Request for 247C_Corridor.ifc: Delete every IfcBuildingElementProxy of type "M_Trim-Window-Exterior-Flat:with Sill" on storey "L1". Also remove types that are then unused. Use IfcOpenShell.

First a look at what the model holds.

```python
import ifcopenshell
import ifcopenshell.util.element

model = ifcopenshell.open("247C_Corridor.ifc")
print(model.schema)
storey = next(s for s in model.by_type("IfcBuildingStorey") if s.Name == "L1")
proxies = [e for e in ifcopenshell.util.element.get_decomposition(storey) if e.is_a("IfcBuildingElementProxy")]
seen = {}
for e in proxies:
    element_type = ifcopenshell.util.element.get_type(e)
    name = element_type.Name if element_type not in (None, e) else None
    seen[name] = seen.get(name, 0) + 1
for name, count in sorted(seen.items(), key=str):
    print(count, "x", name)
```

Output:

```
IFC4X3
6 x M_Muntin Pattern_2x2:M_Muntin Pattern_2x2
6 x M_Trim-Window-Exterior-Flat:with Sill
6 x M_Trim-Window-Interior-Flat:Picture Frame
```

```python
import ifcopenshell
import ifcopenshell.api.root
import ifcopenshell.util.element

model = ifcopenshell.open("247C_Corridor.ifc")

storey = next(s for s in model.by_type("IfcBuildingStorey") if s.Name == "L1")
proxies = [e for e in ifcopenshell.util.element.get_decomposition(storey) if e.is_a("IfcBuildingElementProxy")]
targets = [e for e in proxies if (t := ifcopenshell.util.element.get_type(e)) not in (None, e) and t.Name == "M_Trim-Window-Exterior-Flat:with Sill"]
types = {ifcopenshell.util.element.get_type(e) for e in targets} - {None, *targets}

for e in targets:
    ifcopenshell.api.root.remove_product(model, product=e)
print(len(targets), "removed")

unused = [t for t in types if not ifcopenshell.util.element.get_types(t)]
for t in unused:
    ifcopenshell.api.root.remove_product(model, product=t)
print(len(unused), "unused types removed")

model.write("247C_Corridor_rev.ifc")
```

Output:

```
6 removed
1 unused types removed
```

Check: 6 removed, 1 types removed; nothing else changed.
